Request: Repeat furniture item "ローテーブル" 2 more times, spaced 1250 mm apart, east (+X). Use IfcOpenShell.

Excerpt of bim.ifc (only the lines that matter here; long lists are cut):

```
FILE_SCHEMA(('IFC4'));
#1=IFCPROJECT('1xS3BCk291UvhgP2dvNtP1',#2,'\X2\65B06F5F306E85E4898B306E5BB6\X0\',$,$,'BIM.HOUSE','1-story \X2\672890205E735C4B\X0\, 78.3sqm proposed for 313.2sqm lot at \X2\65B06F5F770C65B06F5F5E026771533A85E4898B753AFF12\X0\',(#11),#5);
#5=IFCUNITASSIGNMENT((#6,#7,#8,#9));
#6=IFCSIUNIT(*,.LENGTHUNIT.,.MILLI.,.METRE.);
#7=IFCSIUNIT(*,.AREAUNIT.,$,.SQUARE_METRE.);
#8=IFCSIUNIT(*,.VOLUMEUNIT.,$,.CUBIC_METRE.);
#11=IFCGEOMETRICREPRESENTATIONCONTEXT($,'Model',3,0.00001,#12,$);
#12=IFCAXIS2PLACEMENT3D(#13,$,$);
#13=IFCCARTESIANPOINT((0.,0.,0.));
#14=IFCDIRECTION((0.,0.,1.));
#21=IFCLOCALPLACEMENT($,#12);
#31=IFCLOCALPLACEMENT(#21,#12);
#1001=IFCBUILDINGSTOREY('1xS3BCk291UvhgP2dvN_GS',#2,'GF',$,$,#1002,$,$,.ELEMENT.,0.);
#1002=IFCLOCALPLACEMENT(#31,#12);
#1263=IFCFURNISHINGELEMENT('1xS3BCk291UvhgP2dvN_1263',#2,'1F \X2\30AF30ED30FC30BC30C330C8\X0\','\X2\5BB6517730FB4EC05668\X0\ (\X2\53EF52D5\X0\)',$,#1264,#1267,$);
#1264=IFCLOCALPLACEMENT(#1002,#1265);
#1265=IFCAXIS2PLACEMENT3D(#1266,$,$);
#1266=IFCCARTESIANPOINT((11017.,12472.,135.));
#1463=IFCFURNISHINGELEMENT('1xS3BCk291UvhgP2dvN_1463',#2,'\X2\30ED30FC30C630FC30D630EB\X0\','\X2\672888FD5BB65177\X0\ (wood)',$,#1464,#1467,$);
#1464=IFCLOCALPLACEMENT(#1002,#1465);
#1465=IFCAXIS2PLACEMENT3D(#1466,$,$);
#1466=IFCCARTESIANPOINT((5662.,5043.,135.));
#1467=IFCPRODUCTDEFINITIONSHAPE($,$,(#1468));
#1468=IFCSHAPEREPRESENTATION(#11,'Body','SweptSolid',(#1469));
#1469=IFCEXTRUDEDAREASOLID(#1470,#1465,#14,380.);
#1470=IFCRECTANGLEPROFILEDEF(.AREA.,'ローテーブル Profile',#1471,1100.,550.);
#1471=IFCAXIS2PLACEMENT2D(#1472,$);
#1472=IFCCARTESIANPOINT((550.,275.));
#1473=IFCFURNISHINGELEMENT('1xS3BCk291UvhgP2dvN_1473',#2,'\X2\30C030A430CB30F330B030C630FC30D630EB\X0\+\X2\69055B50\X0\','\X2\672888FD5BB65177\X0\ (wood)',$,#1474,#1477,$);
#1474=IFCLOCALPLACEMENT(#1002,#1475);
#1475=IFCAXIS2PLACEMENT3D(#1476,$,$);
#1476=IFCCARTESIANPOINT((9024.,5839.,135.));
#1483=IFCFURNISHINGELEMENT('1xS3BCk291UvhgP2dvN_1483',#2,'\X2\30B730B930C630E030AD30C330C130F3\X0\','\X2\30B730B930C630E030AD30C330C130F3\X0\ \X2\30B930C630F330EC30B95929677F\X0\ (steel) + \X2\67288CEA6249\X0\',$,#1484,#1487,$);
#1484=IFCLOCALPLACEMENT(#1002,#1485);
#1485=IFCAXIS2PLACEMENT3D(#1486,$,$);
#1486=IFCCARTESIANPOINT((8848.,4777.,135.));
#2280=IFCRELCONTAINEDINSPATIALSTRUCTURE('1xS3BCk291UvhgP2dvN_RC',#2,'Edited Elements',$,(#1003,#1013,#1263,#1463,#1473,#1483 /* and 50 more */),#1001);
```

```python
import numpy as np
import ifcopenshell
import ifcopenshell.api.geometry
import ifcopenshell.api.root
import ifcopenshell.util.element
import ifcopenshell.util.placement
import ifcopenshell.util.unit

model = ifcopenshell.open("bim.ifc")
unit_scale = ifcopenshell.util.unit.calculate_unit_scale(model)


def reuse_history(source, copy):
    """copy_class also copies each property set's owner history, people and application; keep the originals."""
    for rel in copy.IsDefinedBy:
        if rel.is_a("IfcRelDefinesByProperties") and (history := rel.RelatingPropertyDefinition.OwnerHistory):
            rel.RelatingPropertyDefinition.OwnerHistory = source.OwnerHistory
            ifcopenshell.util.element.remove_deep2(model, history)


source = model.by_id(1463)
base = ifcopenshell.util.placement.get_local_placement(source.ObjectPlacement)
step = np.array([1.0, 0.0, 0.0]) * 1.25 / unit_scale

for i in range(1, 3):
    copy = ifcopenshell.api.root.copy_class(model, product=source)
    copy.Representation = ifcopenshell.util.element.copy_deep(
        model, source.Representation, exclude=["IfcGeometricRepresentationContext", "IfcRepresentationMap"]
    )
    reuse_history(source, copy)
    matrix = base.copy()
    matrix[:3, 3] += i * step
    print("added at", matrix[:3, 3].round(3) + 0.0)
    ifcopenshell.api.geometry.edit_object_placement(model, product=copy, matrix=matrix, is_si=False)

model.write("bim_rev.ifc")
```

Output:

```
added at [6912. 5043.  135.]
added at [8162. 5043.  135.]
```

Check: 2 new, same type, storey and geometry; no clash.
